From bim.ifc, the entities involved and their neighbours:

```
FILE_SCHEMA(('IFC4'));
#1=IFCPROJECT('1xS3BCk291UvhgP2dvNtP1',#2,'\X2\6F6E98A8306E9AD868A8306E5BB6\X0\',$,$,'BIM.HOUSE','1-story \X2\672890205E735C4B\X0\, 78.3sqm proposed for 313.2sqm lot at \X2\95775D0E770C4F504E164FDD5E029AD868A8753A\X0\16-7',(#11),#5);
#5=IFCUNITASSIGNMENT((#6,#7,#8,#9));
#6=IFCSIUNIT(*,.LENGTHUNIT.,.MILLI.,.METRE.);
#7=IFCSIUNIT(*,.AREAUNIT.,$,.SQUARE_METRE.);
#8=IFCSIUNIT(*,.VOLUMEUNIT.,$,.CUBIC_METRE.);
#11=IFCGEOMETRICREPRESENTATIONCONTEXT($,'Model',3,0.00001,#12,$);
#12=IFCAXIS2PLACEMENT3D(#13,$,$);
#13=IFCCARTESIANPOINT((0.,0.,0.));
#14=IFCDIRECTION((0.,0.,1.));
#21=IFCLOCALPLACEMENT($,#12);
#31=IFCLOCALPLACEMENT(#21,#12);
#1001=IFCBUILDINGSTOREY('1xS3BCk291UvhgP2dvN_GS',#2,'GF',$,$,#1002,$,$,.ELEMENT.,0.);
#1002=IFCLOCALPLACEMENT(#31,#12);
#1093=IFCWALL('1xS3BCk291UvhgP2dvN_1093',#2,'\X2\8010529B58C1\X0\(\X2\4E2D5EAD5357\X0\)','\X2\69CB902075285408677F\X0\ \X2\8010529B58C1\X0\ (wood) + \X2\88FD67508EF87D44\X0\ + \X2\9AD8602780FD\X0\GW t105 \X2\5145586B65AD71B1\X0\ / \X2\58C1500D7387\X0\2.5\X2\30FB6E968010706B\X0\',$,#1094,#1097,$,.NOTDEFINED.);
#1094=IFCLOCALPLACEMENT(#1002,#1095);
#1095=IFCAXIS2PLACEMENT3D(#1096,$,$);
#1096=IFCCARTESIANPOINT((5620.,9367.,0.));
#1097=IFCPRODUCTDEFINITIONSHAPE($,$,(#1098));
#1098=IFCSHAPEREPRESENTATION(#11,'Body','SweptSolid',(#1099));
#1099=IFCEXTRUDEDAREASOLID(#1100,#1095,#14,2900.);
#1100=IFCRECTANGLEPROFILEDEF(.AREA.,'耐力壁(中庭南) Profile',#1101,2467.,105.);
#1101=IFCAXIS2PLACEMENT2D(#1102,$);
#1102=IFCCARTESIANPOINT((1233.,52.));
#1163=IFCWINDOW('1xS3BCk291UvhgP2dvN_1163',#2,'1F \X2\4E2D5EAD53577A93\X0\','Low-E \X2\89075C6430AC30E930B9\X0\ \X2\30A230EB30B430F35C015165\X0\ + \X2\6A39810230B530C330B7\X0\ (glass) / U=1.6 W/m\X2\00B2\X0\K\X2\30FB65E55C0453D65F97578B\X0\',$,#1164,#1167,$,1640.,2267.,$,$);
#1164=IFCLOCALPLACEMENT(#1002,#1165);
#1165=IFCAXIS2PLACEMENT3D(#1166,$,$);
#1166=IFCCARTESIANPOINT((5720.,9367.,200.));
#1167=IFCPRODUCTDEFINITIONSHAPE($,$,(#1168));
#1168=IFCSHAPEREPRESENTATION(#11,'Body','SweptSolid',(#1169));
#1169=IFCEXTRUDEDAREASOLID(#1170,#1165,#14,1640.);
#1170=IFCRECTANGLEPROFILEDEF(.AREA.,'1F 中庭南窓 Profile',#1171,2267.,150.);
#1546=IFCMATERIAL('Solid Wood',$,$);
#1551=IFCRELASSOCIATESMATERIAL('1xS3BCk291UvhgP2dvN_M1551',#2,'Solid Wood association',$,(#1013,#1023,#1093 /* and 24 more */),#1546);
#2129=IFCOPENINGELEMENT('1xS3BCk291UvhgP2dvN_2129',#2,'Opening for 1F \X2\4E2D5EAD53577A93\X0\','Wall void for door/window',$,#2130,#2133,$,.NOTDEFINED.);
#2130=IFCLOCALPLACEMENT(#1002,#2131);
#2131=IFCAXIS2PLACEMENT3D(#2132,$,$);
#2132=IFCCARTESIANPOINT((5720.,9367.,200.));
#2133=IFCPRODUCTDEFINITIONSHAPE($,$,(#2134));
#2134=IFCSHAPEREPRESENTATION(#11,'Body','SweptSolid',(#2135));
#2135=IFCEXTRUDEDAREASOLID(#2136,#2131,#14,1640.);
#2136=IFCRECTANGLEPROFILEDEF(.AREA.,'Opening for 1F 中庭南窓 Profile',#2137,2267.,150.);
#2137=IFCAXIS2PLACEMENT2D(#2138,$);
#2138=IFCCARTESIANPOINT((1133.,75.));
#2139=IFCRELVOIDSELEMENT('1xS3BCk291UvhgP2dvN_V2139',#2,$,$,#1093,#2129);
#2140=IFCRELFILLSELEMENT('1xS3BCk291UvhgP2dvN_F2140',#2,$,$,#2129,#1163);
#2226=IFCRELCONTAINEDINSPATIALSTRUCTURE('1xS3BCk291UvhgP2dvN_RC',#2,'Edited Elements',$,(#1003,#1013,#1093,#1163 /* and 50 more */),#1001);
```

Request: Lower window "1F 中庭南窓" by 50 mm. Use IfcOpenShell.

```python
import numpy as np
import ifcopenshell
import ifcopenshell.api.geometry
import ifcopenshell.util.placement
import ifcopenshell.util.unit

model = ifcopenshell.open("bim.ifc")
unit_scale = ifcopenshell.util.unit.calculate_unit_scale(model)

window = model.by_guid("1xS3BCk291UvhgP2dvN_1163")
opening = window.FillsVoids[0].RelatingOpeningElement
dz = -50.0

shift = np.array([0.0, 0.0, dz])
# The window is not placed relative to its opening, so move both.
for product in (opening, window):
    matrix = ifcopenshell.util.placement.get_local_placement(product.ObjectPlacement)
    matrix[:3, 3] += shift
    ifcopenshell.api.geometry.edit_object_placement(model, product=product, matrix=matrix, is_si=False)

print(f"moved by {dz * unit_scale:+.3f} m")

model.write("bim_updated.ifc")
```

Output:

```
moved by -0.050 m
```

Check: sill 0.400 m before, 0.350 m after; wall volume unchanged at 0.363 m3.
